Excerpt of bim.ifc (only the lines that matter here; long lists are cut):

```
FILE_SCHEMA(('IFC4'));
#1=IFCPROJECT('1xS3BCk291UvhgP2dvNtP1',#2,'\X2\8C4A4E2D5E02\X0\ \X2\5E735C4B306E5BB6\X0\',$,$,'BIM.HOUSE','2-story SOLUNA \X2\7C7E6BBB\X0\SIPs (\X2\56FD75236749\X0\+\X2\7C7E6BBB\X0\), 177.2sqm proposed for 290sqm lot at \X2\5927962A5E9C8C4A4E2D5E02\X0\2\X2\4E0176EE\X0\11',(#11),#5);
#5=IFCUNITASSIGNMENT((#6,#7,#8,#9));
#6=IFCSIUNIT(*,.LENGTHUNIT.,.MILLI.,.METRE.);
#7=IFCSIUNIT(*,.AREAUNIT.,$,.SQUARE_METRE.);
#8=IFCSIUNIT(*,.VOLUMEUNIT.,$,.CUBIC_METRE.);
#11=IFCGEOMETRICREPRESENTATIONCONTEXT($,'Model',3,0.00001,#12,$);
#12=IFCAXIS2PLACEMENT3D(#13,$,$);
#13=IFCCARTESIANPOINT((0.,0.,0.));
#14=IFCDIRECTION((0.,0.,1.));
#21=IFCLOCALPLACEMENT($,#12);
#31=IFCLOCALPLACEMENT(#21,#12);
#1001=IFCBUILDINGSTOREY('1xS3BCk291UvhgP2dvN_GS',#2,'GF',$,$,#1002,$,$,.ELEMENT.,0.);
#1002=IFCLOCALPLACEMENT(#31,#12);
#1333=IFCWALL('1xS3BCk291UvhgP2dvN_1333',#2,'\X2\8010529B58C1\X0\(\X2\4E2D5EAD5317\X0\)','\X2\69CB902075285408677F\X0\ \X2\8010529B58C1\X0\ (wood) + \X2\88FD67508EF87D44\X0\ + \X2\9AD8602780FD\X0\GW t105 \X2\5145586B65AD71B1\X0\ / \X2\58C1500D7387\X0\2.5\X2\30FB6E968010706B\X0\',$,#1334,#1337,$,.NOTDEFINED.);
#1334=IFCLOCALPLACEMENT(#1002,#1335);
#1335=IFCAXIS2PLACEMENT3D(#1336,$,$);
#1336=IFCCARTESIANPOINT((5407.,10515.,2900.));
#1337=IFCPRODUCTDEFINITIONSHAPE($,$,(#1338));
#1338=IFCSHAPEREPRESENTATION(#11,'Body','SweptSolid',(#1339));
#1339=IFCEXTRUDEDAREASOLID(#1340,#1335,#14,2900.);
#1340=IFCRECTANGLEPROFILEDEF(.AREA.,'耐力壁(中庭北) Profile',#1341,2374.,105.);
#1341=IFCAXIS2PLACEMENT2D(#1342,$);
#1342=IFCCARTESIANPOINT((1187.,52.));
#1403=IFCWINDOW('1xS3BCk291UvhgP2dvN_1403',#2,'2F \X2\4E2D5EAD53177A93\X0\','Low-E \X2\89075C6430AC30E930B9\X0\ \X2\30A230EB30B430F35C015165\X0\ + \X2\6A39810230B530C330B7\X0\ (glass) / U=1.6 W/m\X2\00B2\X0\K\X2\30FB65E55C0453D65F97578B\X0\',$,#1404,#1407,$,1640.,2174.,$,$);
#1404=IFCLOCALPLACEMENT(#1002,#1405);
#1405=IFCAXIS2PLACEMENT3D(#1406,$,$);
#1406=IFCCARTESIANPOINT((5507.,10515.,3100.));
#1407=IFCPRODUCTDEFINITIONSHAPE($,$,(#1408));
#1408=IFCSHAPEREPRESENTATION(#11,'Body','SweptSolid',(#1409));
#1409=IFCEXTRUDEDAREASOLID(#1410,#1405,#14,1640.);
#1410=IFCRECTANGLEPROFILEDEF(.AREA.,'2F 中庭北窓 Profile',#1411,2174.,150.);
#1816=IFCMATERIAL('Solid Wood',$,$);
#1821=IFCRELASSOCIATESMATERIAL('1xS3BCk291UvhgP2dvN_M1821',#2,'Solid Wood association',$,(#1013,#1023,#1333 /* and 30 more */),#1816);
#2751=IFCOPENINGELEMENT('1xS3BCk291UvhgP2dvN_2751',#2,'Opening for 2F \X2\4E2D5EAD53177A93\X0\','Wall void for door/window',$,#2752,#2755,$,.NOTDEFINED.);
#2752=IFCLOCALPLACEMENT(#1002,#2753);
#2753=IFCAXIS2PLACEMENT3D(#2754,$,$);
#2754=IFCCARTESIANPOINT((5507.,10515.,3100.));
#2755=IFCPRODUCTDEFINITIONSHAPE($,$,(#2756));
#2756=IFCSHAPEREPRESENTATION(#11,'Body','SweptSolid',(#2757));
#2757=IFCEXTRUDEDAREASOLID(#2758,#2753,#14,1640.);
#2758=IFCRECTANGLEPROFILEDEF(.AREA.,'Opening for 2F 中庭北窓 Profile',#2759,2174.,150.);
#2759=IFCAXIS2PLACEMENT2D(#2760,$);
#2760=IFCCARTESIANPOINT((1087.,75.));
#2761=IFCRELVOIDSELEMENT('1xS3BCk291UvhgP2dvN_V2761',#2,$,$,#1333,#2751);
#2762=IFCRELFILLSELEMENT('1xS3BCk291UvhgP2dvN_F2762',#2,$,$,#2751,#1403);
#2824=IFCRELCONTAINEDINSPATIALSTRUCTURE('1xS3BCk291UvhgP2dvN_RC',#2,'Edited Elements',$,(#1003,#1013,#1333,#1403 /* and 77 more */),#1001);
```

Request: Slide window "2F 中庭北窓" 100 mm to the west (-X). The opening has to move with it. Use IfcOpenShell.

```python
import ifcopenshell
import ifcopenshell.api.geometry
import ifcopenshell.util.placement

model = ifcopenshell.open("bim.ifc")

window = model.by_id(1403)
opening = window.FillsVoids[0].RelatingOpeningElement
wall = opening.VoidsElements[0].RelatingBuildingElement

wall_matrix = ifcopenshell.util.placement.get_local_placement(wall.ObjectPlacement)
shift = wall_matrix[:3, 0] * -100.0
before = ifcopenshell.util.placement.get_local_placement(window.ObjectPlacement)[:3, 3].copy()

# The window is not placed relative to its opening, so move both.
for product in (opening, window):
    matrix = ifcopenshell.util.placement.get_local_placement(product.ObjectPlacement)
    matrix[:3, 3] += shift
    ifcopenshell.api.geometry.edit_object_placement(model, product=product, matrix=matrix, is_si=False)

after = ifcopenshell.util.placement.get_local_placement(window.ObjectPlacement)[:3, 3]
print("window moved by", (after - before).round(3) + 0.0)

model.write("bim_rev.ifc")
```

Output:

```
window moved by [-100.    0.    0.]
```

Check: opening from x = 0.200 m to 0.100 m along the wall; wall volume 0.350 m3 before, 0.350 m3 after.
